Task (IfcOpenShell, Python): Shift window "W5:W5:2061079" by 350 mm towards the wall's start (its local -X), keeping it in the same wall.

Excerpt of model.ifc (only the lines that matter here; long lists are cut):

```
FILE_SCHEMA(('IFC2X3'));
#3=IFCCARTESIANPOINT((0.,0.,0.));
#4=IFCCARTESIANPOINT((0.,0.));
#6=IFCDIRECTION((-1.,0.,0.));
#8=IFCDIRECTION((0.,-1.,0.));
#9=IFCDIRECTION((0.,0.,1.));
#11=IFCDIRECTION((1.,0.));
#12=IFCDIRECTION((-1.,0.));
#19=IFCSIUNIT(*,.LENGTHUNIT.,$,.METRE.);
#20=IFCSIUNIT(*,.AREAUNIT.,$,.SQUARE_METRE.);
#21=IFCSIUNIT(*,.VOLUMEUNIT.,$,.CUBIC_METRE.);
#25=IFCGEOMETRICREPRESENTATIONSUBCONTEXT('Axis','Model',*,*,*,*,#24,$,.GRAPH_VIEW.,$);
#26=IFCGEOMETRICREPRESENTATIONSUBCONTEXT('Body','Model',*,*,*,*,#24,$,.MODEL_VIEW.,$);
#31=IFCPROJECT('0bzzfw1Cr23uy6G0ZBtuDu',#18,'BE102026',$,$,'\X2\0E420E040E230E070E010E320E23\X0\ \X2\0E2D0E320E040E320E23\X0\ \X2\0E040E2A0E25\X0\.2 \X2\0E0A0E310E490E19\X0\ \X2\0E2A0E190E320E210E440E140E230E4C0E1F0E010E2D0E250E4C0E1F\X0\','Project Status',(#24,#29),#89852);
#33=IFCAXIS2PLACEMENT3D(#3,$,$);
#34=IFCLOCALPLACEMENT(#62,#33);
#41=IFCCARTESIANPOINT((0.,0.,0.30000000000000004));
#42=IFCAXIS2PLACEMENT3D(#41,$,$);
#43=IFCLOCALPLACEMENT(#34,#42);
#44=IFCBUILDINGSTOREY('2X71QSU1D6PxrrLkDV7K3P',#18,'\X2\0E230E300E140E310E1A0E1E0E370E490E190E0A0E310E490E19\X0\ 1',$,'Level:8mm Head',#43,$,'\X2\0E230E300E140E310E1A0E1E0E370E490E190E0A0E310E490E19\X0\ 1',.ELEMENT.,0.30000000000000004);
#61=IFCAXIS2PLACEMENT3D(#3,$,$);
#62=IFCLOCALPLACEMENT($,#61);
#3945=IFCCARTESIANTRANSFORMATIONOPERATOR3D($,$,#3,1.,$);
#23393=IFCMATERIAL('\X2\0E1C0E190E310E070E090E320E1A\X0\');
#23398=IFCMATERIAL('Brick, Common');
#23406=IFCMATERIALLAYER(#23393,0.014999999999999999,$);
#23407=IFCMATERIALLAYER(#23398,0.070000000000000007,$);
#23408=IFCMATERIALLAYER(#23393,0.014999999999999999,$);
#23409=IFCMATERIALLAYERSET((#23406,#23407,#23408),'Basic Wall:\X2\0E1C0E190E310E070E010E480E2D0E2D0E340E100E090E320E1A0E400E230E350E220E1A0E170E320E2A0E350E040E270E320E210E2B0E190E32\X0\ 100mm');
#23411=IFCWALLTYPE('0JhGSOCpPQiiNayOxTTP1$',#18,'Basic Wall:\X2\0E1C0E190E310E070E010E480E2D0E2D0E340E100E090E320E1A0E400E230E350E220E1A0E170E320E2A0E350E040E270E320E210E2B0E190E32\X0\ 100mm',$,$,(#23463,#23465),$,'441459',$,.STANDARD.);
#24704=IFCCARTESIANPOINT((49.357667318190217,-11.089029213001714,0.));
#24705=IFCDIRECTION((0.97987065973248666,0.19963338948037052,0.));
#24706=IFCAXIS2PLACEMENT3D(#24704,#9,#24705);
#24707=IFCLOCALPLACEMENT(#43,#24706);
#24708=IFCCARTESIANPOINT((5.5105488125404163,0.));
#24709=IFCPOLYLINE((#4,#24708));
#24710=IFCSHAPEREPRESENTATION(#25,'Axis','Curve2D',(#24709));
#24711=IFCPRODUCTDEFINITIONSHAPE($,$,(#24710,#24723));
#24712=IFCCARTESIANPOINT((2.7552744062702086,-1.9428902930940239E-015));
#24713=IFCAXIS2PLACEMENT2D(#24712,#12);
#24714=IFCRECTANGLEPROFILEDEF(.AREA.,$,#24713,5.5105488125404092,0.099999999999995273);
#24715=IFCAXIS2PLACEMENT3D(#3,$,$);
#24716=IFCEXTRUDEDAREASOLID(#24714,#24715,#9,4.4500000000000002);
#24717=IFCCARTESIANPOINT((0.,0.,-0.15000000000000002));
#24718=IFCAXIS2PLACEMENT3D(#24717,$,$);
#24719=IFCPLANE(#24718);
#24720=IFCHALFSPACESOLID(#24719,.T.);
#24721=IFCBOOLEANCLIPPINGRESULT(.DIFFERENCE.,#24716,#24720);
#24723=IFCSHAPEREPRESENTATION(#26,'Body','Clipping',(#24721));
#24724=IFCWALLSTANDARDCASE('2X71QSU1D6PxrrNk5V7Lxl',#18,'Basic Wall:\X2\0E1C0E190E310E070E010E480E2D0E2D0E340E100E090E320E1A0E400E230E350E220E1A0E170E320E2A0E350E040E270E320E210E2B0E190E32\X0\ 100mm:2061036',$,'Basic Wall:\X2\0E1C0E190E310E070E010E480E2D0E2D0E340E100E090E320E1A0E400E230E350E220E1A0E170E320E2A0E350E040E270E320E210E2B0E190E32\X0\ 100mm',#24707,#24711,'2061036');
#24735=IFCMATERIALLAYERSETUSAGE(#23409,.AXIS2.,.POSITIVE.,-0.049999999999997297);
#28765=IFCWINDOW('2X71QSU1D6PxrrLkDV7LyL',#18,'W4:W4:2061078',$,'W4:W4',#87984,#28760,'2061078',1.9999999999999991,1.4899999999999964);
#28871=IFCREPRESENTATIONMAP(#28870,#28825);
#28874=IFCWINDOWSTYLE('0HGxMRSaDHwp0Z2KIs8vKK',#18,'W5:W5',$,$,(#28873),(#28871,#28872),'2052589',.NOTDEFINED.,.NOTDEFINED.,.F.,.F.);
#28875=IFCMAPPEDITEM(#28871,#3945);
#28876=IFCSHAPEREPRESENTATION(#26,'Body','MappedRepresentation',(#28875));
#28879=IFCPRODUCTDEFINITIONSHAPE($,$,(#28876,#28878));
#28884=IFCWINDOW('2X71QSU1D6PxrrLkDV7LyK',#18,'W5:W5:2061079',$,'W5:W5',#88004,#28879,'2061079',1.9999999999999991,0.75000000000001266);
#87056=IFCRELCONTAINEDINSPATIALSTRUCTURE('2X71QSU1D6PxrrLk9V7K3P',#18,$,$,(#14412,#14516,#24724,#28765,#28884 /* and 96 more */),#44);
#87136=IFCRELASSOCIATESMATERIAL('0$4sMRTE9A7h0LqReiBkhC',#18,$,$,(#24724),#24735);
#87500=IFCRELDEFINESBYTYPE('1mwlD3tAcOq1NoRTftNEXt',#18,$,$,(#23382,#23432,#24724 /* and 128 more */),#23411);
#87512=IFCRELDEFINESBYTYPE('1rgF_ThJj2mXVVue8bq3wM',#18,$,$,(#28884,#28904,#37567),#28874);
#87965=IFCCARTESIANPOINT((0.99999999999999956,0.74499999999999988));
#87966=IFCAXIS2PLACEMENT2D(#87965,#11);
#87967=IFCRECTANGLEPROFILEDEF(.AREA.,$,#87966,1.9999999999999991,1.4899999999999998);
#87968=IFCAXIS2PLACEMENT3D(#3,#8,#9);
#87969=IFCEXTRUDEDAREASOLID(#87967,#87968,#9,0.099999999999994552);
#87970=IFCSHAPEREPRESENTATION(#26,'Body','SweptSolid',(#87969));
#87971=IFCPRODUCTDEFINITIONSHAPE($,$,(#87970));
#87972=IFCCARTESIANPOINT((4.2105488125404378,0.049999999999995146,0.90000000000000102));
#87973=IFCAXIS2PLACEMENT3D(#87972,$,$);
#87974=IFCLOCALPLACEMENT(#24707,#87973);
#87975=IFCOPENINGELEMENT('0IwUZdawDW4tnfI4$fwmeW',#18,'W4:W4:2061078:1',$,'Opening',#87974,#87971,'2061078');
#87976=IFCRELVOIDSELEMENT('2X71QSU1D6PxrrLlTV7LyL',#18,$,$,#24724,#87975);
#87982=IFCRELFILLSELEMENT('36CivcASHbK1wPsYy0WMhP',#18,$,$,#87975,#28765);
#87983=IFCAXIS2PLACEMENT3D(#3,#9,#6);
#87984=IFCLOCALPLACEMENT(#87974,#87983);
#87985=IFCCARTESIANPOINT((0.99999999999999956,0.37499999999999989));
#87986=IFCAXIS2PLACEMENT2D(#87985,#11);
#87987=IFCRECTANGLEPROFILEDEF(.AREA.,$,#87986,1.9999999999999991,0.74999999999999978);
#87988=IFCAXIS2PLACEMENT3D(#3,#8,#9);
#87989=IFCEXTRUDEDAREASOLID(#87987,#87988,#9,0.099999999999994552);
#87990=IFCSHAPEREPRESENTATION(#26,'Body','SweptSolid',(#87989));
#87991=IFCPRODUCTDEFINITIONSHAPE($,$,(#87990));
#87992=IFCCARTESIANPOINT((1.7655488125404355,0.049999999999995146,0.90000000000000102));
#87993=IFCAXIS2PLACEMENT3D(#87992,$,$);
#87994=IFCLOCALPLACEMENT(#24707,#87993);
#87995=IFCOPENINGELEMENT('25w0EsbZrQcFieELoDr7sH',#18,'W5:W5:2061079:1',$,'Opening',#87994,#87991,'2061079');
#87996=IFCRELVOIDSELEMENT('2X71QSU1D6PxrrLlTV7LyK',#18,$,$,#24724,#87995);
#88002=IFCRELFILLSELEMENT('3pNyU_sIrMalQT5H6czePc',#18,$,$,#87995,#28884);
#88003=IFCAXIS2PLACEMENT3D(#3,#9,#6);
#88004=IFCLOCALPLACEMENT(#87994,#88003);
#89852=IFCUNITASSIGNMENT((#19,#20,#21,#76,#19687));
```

```python
import ifcopenshell
import ifcopenshell.api.geometry
import ifcopenshell.util.placement

model = ifcopenshell.open("model.ifc")

window = model.by_guid("2X71QSU1D6PxrrLkDV7LyK")
opening = window.FillsVoids[0].RelatingOpeningElement
wall = opening.VoidsElements[0].RelatingBuildingElement

wall_matrix = ifcopenshell.util.placement.get_local_placement(wall.ObjectPlacement)
shift = wall_matrix[:3, 0] * -0.35
before = ifcopenshell.util.placement.get_local_placement(window.ObjectPlacement)[:3, 3].copy()

# The window is placed relative to its opening, so it follows when the opening moves.
matrix = ifcopenshell.util.placement.get_local_placement(opening.ObjectPlacement)
matrix[:3, 3] += shift
ifcopenshell.api.geometry.edit_object_placement(
    model, product=opening, matrix=matrix, is_si=False, should_transform_children=True
)

after = ifcopenshell.util.placement.get_local_placement(window.ObjectPlacement)[:3, 3]
print("window moved by", (after - before).round(3) + 0.0)

model.write("model_edited.ifc")
```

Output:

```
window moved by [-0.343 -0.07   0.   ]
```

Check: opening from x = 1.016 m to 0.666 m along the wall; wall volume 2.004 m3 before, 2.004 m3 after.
